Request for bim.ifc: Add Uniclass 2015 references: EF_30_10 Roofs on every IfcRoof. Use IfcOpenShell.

First a look at what the model holds.

```python
import ifcopenshell

model = ifcopenshell.open("bim.ifc")
print(model.schema)
print("classifications:", [c.Name for c in model.by_type("IfcClassification")])
for ifc_class in ("IfcDoor", "IfcRoof", "IfcStair", "IfcWall", "IfcWindow"):
    print(ifc_class, len(model.by_type(ifc_class)))
```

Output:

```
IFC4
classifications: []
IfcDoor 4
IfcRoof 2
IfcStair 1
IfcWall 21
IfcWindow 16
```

```python
import ifcopenshell
import ifcopenshell.api.classification

model = ifcopenshell.open("bim.ifc")

system = ifcopenshell.api.classification.add_classification(model, classification="Uniclass 2015")

codes = {
    "IfcRoof": ("EF_30_10", "Roofs"),
}
for ifc_class, (code, name) in codes.items():
    products = model.by_type(ifc_class)
    ifcopenshell.api.classification.add_reference(
        model, products=products, classification=system, identification=code, name=name
    )
    print(code, len(products))

model.write("bim_edited.ifc")
```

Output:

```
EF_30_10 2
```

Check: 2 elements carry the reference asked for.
